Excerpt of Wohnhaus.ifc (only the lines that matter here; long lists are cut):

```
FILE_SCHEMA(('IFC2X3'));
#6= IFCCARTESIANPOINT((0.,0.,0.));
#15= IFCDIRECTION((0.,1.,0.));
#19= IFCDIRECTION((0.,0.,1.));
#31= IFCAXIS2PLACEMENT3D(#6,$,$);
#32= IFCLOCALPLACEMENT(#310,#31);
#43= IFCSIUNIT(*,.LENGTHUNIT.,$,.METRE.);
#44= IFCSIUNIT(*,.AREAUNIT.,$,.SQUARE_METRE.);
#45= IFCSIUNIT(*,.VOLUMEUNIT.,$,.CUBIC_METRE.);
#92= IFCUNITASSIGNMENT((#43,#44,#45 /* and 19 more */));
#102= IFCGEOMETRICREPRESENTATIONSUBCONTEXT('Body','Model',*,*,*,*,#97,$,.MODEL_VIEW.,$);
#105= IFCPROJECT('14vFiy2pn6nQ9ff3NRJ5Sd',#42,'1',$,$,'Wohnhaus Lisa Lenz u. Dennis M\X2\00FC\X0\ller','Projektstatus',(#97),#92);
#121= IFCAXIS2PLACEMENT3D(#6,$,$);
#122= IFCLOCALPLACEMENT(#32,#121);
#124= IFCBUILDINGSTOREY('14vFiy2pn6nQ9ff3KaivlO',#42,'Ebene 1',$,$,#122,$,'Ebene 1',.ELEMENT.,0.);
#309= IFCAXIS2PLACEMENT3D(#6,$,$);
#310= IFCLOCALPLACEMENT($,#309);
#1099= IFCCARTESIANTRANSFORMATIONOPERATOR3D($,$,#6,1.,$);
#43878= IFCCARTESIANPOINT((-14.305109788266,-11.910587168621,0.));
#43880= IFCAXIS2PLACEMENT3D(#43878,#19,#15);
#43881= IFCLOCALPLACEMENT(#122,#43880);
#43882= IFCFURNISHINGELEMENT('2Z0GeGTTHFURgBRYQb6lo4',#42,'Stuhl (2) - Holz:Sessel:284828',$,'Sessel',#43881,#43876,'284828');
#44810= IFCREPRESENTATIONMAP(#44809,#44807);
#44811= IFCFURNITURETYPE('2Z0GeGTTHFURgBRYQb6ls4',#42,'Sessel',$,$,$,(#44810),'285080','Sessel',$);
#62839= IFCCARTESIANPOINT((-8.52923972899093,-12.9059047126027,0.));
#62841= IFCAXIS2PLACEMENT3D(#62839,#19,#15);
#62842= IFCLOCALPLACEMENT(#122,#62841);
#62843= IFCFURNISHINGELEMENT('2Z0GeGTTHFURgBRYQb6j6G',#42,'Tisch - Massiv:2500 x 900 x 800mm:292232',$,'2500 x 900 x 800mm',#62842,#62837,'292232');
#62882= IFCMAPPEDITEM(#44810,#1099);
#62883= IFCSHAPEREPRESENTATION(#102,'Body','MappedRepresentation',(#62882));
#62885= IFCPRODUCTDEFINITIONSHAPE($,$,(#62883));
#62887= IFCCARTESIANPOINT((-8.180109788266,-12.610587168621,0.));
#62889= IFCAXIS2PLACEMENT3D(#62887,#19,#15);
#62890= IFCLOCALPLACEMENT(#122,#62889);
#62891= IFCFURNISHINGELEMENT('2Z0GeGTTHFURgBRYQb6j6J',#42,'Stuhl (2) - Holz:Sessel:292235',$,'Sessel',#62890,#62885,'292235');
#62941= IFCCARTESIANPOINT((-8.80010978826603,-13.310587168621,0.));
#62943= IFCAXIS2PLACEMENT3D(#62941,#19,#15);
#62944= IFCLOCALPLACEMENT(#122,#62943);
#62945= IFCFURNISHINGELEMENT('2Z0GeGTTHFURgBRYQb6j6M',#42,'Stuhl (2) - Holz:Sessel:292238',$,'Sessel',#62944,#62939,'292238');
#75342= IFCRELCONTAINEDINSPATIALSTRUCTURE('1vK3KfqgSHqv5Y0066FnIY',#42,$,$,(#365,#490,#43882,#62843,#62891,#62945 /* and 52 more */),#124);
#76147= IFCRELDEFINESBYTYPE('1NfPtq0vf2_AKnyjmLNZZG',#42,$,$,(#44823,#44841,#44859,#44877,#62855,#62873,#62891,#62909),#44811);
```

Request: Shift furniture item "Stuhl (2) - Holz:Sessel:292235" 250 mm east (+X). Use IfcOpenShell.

```python
import ifcopenshell
import ifcopenshell.api.geometry
import ifcopenshell.util.placement
import ifcopenshell.util.unit

model = ifcopenshell.open("Wohnhaus.ifc")
unit_scale = ifcopenshell.util.unit.calculate_unit_scale(model)

item = model.by_guid("2Z0GeGTTHFURgBRYQb6j6J")
matrix = ifcopenshell.util.placement.get_local_placement(item.ObjectPlacement)
matrix[0, 3] += 0.25 / unit_scale
ifcopenshell.api.geometry.edit_object_placement(model, product=item, matrix=matrix, is_si=False)

print(ifcopenshell.util.placement.get_local_placement(item.ObjectPlacement).round(3) + 0.0)

model.write("Wohnhaus_edited.ifc")
```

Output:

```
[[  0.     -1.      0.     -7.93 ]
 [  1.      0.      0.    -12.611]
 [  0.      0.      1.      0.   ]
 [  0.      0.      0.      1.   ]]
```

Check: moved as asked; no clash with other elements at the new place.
